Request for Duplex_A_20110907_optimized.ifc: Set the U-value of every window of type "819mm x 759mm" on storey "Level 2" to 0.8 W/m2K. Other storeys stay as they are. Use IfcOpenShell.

First a look at what the model holds.

```python
import ifcopenshell
import ifcopenshell.util.element

model = ifcopenshell.open("Duplex_A_20110907_optimized.ifc")
print(model.schema)
storey = next(s for s in model.by_type("IfcBuildingStorey") if s.Name == "Level 2")
windows = [e for e in ifcopenshell.util.element.get_decomposition(storey) if e.is_a("IfcWindow")]
seen = {}
for e in windows:
    element_type = ifcopenshell.util.element.get_type(e)
    key = (element_type.Name if element_type != e and element_type else None, ifcopenshell.util.element.get_pset(e, "Pset_WindowCommon", "ThermalTransmittance"))
    seen[key] = seen.get(key, 0) + 1
for (name, value), count in sorted(seen.items(), key=str):
    print(count, "x", name, "|", value)
```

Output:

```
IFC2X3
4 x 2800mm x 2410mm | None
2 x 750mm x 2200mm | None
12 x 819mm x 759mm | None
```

```python
import ifcopenshell
import ifcopenshell.api.pset
import ifcopenshell.util.element

model = ifcopenshell.open("Duplex_A_20110907_optimized.ifc")

storey = next(s for s in model.by_type("IfcBuildingStorey") if s.Name == "Level 2")
windows = [e for e in ifcopenshell.util.element.get_decomposition(storey) if e.is_a("IfcWindow")]

count = 0
for e in windows:
    element_type = ifcopenshell.util.element.get_type(e)
    if element_type in (None, e) or element_type.Name != "819mm x 759mm":
        continue
    # add_pset returns the element's existing set when there is one.
    pset = ifcopenshell.api.pset.add_pset(model, product=e, name="Pset_WindowCommon")
    ifcopenshell.api.pset.edit_pset(model, pset=pset, properties={"ThermalTransmittance": 0.8})
    count += 1

print(count, "windows updated")

model.write("Duplex_A_20110907_optimized_edited.ifc")
```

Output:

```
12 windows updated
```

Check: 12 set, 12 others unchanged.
